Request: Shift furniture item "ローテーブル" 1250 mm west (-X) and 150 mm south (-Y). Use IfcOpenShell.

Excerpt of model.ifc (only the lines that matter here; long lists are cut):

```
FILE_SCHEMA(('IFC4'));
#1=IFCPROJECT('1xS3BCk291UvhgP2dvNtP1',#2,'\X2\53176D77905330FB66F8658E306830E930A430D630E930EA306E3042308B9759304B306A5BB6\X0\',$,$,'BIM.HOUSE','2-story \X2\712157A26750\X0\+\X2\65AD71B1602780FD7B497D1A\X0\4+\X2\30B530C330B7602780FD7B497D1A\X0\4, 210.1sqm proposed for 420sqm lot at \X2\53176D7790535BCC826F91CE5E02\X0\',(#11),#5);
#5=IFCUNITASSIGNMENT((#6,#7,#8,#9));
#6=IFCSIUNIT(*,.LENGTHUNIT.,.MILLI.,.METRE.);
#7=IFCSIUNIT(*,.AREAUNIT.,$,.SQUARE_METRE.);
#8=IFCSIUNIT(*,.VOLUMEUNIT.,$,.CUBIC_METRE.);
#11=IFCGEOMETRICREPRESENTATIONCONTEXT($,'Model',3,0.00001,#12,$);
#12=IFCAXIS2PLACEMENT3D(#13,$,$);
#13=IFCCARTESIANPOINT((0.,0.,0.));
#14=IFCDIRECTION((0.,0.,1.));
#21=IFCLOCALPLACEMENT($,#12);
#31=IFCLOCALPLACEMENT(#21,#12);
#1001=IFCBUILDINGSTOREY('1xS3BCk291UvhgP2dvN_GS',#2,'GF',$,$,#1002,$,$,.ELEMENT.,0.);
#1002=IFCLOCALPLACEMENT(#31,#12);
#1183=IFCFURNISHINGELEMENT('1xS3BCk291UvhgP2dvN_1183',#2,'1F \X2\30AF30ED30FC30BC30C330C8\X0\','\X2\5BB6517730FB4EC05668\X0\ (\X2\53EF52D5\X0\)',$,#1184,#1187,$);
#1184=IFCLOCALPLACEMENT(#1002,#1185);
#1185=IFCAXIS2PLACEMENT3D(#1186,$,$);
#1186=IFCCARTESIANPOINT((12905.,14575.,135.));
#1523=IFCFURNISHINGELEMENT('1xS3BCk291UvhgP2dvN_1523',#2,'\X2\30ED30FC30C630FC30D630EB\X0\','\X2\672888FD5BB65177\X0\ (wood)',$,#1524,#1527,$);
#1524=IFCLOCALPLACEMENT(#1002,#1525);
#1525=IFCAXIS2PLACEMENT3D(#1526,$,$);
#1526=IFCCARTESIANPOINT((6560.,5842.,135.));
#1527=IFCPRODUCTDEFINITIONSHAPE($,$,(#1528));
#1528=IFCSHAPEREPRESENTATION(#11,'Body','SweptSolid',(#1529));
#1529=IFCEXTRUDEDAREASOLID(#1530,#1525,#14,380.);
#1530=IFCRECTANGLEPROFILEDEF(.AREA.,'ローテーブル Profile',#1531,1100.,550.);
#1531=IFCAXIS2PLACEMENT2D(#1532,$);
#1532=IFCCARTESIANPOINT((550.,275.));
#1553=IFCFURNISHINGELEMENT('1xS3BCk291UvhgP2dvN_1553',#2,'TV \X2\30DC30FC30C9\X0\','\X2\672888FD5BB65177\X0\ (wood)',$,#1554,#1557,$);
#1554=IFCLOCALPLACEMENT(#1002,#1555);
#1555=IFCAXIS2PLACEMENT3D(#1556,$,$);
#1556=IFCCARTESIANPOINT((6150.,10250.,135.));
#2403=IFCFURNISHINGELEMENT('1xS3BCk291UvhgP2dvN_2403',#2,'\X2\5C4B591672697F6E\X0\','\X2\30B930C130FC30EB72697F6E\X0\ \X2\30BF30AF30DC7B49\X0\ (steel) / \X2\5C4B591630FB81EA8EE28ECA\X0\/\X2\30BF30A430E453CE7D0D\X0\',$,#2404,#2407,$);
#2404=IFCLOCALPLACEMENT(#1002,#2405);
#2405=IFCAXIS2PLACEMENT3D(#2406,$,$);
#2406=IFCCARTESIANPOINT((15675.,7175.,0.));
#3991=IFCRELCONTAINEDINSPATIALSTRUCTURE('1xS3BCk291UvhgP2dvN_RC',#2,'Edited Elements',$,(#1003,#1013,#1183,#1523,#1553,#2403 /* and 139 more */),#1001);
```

```python
import ifcopenshell
import ifcopenshell.api.geometry
import ifcopenshell.util.placement
import ifcopenshell.util.unit

model = ifcopenshell.open("model.ifc")
unit_scale = ifcopenshell.util.unit.calculate_unit_scale(model)

item = model.by_id(1523)
matrix = ifcopenshell.util.placement.get_local_placement(item.ObjectPlacement)
matrix[0, 3] -= 1.25 / unit_scale
matrix[1, 3] -= 0.15 / unit_scale
ifcopenshell.api.geometry.edit_object_placement(model, product=item, matrix=matrix, is_si=False)

print(ifcopenshell.util.placement.get_local_placement(item.ObjectPlacement).round(3) + 0.0)

model.write("model_v2.ifc")
```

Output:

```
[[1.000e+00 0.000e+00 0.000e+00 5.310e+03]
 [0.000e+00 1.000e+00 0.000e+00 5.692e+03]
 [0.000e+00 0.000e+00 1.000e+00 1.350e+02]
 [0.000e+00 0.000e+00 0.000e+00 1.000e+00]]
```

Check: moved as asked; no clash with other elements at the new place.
